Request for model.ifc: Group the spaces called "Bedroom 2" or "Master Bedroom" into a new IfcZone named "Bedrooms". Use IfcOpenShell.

First a look at what the model holds.

```python
import ifcopenshell

model = ifcopenshell.open("model.ifc")
print(model.schema)
seen = {}
for space in model.by_type("IfcSpace"):
    seen[space.LongName] = seen.get(space.LongName, 0) + 1
for name, count in sorted(seen.items(), key=str):
    print(count, "x", name)
print("zones:", [z.Name for z in model.by_type("IfcZone")][:20])
```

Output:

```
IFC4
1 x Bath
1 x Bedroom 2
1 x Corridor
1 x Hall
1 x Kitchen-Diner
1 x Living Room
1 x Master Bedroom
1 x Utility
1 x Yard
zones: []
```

```python
import ifcopenshell
import ifcopenshell.api.group
import ifcopenshell.api.root

model = ifcopenshell.open("model.ifc")

names = {"Bedroom 2", "Master Bedroom"}
spaces = [s for s in model.by_type("IfcSpace") if s.LongName in names]

zone = ifcopenshell.api.root.create_entity(model, ifc_class="IfcZone", name="Bedrooms")
ifcopenshell.api.group.assign_group(model, products=spaces, group=zone)
print(len(spaces), "spaces in", zone.Name)

model.write("model-out.ifc")
```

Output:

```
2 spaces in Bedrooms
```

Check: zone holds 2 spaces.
